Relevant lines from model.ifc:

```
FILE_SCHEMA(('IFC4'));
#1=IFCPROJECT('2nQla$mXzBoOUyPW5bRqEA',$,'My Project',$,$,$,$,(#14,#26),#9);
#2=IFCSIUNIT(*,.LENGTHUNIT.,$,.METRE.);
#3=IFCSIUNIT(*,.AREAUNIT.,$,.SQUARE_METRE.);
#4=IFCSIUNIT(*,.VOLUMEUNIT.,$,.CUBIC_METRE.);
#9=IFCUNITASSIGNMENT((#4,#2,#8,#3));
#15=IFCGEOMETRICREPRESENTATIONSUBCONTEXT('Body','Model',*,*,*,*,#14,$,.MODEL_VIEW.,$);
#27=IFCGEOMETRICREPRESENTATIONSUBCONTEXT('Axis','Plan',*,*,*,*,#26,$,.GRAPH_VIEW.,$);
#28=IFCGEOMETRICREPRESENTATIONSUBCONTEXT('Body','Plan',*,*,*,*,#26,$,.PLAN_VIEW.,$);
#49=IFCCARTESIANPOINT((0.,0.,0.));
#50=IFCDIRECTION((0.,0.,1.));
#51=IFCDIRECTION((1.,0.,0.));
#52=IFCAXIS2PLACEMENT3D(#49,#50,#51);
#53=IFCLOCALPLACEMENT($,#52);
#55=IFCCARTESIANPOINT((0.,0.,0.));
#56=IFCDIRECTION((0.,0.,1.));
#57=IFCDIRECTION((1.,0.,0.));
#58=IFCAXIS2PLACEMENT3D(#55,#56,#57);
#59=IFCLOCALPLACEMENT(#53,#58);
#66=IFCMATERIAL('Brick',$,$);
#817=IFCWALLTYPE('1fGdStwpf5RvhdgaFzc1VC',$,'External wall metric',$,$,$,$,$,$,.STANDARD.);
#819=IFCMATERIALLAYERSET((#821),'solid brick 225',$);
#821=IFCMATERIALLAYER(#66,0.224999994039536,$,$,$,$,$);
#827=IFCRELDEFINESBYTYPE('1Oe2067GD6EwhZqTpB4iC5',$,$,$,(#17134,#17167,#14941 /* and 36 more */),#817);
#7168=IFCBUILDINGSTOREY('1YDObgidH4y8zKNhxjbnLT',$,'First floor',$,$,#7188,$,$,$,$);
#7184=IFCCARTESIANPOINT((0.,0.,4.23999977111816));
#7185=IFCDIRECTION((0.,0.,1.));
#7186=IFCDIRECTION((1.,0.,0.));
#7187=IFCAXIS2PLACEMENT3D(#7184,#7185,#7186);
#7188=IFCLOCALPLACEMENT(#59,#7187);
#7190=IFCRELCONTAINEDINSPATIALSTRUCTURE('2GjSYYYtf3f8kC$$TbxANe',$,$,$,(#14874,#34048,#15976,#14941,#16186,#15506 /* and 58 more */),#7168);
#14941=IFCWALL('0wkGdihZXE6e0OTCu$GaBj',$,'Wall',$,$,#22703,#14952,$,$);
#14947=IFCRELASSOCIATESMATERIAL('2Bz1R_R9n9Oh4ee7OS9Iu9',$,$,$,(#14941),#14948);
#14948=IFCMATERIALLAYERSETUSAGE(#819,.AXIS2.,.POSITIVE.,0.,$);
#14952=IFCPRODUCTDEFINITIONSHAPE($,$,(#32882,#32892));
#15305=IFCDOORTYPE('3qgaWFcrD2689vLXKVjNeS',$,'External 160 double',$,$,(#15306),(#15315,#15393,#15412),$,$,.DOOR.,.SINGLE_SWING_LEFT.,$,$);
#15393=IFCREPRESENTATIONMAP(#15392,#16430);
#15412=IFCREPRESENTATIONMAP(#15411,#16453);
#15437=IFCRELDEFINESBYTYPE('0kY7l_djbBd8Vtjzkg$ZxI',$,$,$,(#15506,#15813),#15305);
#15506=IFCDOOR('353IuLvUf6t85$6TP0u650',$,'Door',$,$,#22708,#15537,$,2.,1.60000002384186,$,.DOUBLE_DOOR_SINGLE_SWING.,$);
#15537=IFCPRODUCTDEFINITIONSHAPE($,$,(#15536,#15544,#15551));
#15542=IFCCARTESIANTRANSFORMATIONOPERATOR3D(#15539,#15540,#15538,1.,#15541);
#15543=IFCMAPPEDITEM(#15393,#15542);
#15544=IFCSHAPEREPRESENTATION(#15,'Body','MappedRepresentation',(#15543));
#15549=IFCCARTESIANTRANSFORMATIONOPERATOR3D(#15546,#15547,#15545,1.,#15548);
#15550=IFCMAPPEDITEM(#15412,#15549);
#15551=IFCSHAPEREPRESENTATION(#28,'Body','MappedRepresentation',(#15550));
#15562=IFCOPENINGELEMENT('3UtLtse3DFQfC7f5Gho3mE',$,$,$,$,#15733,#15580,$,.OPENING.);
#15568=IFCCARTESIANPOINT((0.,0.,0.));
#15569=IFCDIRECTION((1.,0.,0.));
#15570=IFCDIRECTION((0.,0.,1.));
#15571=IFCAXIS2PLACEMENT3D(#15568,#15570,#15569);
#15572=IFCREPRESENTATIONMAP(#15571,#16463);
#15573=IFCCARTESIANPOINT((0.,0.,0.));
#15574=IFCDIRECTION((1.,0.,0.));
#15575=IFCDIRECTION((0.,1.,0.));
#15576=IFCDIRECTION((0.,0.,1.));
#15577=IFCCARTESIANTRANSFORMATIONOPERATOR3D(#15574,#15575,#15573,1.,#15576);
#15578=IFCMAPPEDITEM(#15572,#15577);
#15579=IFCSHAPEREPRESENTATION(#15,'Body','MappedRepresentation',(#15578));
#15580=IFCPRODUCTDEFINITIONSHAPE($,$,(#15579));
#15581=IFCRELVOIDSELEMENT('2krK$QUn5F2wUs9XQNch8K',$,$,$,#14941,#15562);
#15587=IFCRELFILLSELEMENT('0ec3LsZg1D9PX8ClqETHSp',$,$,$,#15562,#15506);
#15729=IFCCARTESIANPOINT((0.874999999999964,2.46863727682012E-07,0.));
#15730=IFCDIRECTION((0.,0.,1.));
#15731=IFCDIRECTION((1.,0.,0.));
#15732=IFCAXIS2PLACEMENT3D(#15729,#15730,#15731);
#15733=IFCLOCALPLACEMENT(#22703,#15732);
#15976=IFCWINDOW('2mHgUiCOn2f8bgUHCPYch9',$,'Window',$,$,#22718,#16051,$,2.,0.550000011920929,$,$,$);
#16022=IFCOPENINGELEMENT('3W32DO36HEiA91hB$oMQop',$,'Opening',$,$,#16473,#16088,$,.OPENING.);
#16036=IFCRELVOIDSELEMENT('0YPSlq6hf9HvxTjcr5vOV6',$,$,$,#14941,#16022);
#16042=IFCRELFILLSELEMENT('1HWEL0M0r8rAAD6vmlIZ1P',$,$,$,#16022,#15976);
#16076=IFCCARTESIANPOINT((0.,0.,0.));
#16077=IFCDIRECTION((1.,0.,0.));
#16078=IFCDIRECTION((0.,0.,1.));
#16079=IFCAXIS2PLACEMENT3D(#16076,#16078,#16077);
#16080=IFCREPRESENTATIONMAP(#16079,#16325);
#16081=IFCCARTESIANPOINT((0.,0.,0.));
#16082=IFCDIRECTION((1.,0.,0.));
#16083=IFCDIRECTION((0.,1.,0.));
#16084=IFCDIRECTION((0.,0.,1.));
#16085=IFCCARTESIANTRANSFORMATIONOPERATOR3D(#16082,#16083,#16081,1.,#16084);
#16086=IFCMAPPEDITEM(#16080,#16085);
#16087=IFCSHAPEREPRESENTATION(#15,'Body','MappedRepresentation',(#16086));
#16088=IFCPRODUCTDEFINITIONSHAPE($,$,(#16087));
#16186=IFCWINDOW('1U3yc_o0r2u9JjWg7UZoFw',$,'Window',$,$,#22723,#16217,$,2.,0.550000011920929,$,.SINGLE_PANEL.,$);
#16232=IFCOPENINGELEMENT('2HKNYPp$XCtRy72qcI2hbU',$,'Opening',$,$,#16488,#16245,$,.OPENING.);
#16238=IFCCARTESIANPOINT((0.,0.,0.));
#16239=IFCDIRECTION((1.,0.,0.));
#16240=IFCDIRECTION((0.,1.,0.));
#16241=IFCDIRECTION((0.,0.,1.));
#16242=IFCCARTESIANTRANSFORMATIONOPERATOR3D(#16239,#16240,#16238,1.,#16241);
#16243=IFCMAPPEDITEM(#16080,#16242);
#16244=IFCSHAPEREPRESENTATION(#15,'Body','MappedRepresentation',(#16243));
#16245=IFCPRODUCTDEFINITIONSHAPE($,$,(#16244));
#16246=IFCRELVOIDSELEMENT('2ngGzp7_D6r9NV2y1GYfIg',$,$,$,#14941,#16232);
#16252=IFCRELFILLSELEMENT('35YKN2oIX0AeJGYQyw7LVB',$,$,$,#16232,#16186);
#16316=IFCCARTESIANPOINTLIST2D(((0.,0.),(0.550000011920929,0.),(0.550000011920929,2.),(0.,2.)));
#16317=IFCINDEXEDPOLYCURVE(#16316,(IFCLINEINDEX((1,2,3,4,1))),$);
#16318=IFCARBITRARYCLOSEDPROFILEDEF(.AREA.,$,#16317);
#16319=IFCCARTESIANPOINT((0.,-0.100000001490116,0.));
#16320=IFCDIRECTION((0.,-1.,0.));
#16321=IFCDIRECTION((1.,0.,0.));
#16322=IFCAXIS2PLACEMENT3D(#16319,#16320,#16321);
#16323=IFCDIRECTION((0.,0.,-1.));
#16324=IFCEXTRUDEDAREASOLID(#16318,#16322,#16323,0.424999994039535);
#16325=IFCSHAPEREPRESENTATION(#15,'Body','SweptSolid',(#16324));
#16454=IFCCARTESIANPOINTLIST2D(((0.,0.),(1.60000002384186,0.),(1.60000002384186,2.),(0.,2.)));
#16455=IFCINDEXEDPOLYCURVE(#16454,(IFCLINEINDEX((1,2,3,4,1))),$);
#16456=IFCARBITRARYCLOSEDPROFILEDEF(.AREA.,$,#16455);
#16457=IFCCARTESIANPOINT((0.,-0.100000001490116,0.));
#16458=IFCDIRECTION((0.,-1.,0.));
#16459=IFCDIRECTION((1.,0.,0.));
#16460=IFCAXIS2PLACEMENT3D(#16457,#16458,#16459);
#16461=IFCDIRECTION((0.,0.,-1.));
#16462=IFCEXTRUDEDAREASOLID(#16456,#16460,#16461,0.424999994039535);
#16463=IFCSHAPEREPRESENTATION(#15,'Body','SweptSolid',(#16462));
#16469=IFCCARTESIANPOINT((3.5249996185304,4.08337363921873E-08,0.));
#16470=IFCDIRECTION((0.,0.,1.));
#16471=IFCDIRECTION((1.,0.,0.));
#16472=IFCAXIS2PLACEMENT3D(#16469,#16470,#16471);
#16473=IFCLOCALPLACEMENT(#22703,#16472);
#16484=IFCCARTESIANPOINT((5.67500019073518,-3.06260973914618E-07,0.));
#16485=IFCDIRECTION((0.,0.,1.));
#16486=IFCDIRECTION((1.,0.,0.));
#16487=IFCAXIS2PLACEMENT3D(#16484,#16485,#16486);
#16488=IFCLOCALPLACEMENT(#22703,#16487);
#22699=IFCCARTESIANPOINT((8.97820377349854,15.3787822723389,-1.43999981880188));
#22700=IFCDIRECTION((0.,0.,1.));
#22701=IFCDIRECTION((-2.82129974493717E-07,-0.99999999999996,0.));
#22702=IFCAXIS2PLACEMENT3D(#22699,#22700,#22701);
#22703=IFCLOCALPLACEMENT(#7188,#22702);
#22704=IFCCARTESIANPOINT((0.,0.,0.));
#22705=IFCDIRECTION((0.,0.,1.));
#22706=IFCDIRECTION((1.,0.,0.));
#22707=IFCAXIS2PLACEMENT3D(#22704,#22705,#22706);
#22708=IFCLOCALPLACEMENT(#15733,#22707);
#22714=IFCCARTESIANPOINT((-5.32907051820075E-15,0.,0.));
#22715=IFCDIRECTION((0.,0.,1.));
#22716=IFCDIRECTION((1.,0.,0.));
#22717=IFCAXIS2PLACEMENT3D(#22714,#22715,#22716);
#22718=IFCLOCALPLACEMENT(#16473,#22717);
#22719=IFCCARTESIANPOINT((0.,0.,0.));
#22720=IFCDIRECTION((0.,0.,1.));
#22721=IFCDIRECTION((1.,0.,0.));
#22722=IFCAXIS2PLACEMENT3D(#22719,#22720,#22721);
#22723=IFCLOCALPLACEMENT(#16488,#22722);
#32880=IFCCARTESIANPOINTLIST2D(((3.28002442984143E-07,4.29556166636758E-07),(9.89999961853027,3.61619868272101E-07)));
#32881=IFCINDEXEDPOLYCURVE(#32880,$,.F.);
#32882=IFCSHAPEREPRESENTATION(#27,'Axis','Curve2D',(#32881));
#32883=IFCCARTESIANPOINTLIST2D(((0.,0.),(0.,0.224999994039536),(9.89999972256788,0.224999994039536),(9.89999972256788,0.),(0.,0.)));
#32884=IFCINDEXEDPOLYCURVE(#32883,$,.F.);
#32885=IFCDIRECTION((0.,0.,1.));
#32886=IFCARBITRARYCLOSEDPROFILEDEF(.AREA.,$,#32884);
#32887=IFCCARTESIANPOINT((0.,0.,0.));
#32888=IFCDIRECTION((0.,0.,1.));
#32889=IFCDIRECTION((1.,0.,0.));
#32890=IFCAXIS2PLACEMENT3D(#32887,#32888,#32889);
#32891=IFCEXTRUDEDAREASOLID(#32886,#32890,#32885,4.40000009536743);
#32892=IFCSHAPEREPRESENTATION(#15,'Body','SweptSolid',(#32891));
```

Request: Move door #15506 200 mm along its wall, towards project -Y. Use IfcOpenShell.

```python
import ifcopenshell
import ifcopenshell.api.geometry
import ifcopenshell.util.placement
import ifcopenshell.util.unit

model = ifcopenshell.open("model.ifc")
unit_scale = ifcopenshell.util.unit.calculate_unit_scale(model)

door = model.by_guid("353IuLvUf6t85$6TP0u650")
opening = door.FillsVoids[0].RelatingOpeningElement
wall = opening.VoidsElements[0].RelatingBuildingElement

wall_matrix = ifcopenshell.util.placement.get_local_placement(wall.ObjectPlacement)
shift = wall_matrix[:3, 0] * 0.2 / unit_scale
before = ifcopenshell.util.placement.get_local_placement(door.ObjectPlacement)[:3, 3].copy()

# The door is placed relative to its opening, so it follows when the opening moves.
matrix = ifcopenshell.util.placement.get_local_placement(opening.ObjectPlacement)
matrix[:3, 3] += shift
ifcopenshell.api.geometry.edit_object_placement(
    model, product=opening, matrix=matrix, is_si=False, should_transform_children=True
)

after = ifcopenshell.util.placement.get_local_placement(door.ObjectPlacement)[:3, 3]
print("door moved by", (after - before).round(3) + 0.0)

model.write("model_edited.ifc")
```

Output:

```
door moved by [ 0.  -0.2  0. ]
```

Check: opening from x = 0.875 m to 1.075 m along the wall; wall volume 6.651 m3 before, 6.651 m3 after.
